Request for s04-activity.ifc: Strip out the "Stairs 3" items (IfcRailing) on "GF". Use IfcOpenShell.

First a look at what the model holds.

```python
import ifcopenshell
import ifcopenshell.util.element

model = ifcopenshell.open("s04-activity.ifc")
print(model.schema)
storey = next(s for s in model.by_type("IfcBuildingStorey") if s.Name == "GF")
railings = [e for e in ifcopenshell.util.element.get_decomposition(storey) if e.is_a("IfcRailing")]
seen = {}
for e in railings:
    element_type = ifcopenshell.util.element.get_type(e)
    name = element_type.Name if element_type not in (None, e) else None
    seen[name] = seen.get(name, 0) + 1
for name, count in sorted(seen.items(), key=str):
    print(count, "x", name)
```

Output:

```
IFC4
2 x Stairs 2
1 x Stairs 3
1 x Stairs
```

```python
import ifcopenshell
import ifcopenshell.api.root
import ifcopenshell.util.element

model = ifcopenshell.open("s04-activity.ifc")

storey = next(s for s in model.by_type("IfcBuildingStorey") if s.Name == "GF")
railings = [e for e in ifcopenshell.util.element.get_decomposition(storey) if e.is_a("IfcRailing")]
targets = [e for e in railings if (t := ifcopenshell.util.element.get_type(e)) not in (None, e) and t.Name == "Stairs 3"]

for e in targets:
    ifcopenshell.api.root.remove_product(model, product=e)
print(len(targets), "removed")

model.write("s04-activity_rev.ifc")
```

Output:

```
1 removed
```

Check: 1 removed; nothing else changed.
